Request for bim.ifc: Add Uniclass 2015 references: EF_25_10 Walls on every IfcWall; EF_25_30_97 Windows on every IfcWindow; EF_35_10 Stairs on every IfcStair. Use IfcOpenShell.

First a look at what the model holds.

```python
import ifcopenshell

model = ifcopenshell.open("bim.ifc")
print(model.schema)
print("classifications:", [c.Name for c in model.by_type("IfcClassification")])
for ifc_class in ("IfcDoor", "IfcRoof", "IfcStair", "IfcWall", "IfcWindow"):
    print(ifc_class, len(model.by_type(ifc_class)))
```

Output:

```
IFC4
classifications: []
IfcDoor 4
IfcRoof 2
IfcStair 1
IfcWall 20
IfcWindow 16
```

```python
import ifcopenshell
import ifcopenshell.api.classification

model = ifcopenshell.open("bim.ifc")

system = ifcopenshell.api.classification.add_classification(model, classification="Uniclass 2015")

codes = {
    "IfcWall": ("EF_25_10", "Walls"),
    "IfcWindow": ("EF_25_30_97", "Windows"),
    "IfcStair": ("EF_35_10", "Stairs"),
}
for ifc_class, (code, name) in codes.items():
    products = model.by_type(ifc_class)
    ifcopenshell.api.classification.add_reference(
        model, products=products, classification=system, identification=code, name=name
    )
    print(code, len(products))

model.write("bim_v2.ifc")
```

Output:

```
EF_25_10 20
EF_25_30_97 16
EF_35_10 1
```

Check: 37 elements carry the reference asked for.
